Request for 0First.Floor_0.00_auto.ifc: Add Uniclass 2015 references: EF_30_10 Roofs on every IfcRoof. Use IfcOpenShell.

First a look at what the model holds.

```python
import ifcopenshell

model = ifcopenshell.open("0First.Floor_0.00_auto.ifc")
print(model.schema)
print("classifications:", [c.Name for c in model.by_type("IfcClassification")])
for ifc_class in ("IfcDoor", "IfcRoof", "IfcStair", "IfcWall", "IfcWindow"):
    print(ifc_class, len(model.by_type(ifc_class)))
```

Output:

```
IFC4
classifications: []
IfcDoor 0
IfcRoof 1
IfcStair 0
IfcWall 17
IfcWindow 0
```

```python
import ifcopenshell
import ifcopenshell.api.classification

model = ifcopenshell.open("0First.Floor_0.00_auto.ifc")

system = ifcopenshell.api.classification.add_classification(model, classification="Uniclass 2015")

codes = {
    "IfcRoof": ("EF_30_10", "Roofs"),
}
for ifc_class, (code, name) in codes.items():
    products = model.by_type(ifc_class)
    ifcopenshell.api.classification.add_reference(
        model, products=products, classification=system, identification=code, name=name
    )
    print(code, len(products))

model.write("0First.Floor_0.00_auto_edited.ifc")
```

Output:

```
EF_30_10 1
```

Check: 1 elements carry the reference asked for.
